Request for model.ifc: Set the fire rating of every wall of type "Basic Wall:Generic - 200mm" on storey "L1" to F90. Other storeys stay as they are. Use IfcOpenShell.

First a look at what the model holds.

```python
import ifcopenshell
import ifcopenshell.util.element

model = ifcopenshell.open("model.ifc")
print(model.schema)
storey = next(s for s in model.by_type("IfcBuildingStorey") if s.Name == "L1")
walls = [e for e in ifcopenshell.util.element.get_decomposition(storey) if e.is_a("IfcWall")]
seen = {}
for e in walls:
    element_type = ifcopenshell.util.element.get_type(e)
    key = (element_type.Name if element_type != e and element_type else None, ifcopenshell.util.element.get_pset(e, "Pset_WallCommon", "FireRating"))
    seen[key] = seen.get(key, 0) + 1
for (name, value), count in sorted(seen.items(), key=str):
    print(count, "x", name, "|", value)
```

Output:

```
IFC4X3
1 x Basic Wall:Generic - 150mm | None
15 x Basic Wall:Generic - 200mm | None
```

```python
import ifcopenshell
import ifcopenshell.api.pset
import ifcopenshell.util.element

model = ifcopenshell.open("model.ifc")

storey = next(s for s in model.by_type("IfcBuildingStorey") if s.Name == "L1")
walls = [e for e in ifcopenshell.util.element.get_decomposition(storey) if e.is_a("IfcWall")]

count = 0
for e in walls:
    element_type = ifcopenshell.util.element.get_type(e)
    if element_type in (None, e) or element_type.Name != "Basic Wall:Generic - 200mm":
        continue
    # add_pset returns the element's existing set when there is one.
    pset = ifcopenshell.api.pset.add_pset(model, product=e, name="Pset_WallCommon")
    ifcopenshell.api.pset.edit_pset(model, pset=pset, properties={"FireRating": "F90"})
    count += 1

print(count, "walls updated")

model.write("model_updated.ifc")
```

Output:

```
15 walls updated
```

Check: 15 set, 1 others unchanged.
